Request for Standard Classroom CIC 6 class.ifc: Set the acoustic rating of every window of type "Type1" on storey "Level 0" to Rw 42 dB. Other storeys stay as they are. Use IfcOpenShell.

First a look at what the model holds.

```python
import ifcopenshell
import ifcopenshell.util.element

model = ifcopenshell.open("Standard Classroom CIC 6 class.ifc")
print(model.schema)
storey = next(s for s in model.by_type("IfcBuildingStorey") if s.Name == "Level 0")
windows = [e for e in ifcopenshell.util.element.get_decomposition(storey) if e.is_a("IfcWindow")]
seen = {}
for e in windows:
    element_type = ifcopenshell.util.element.get_type(e)
    key = (element_type.Name if element_type != e and element_type else None, ifcopenshell.util.element.get_pset(e, "Pset_WindowCommon", "AcousticRating"))
    seen[key] = seen.get(key, 0) + 1
for (name, value), count in sorted(seen.items(), key=str):
    print(count, "x", name, "|", value)
```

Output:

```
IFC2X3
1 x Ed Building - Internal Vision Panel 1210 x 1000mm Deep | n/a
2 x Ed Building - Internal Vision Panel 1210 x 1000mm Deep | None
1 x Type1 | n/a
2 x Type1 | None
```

```python
import ifcopenshell
import ifcopenshell.api.pset
import ifcopenshell.util.element

model = ifcopenshell.open("Standard Classroom CIC 6 class.ifc")

storey = next(s for s in model.by_type("IfcBuildingStorey") if s.Name == "Level 0")
windows = [e for e in ifcopenshell.util.element.get_decomposition(storey) if e.is_a("IfcWindow")]

count = 0
for e in windows:
    element_type = ifcopenshell.util.element.get_type(e)
    if element_type in (None, e) or element_type.Name != "Type1":
        continue
    # add_pset returns the element's existing set when there is one.
    pset = ifcopenshell.api.pset.add_pset(model, product=e, name="Pset_WindowCommon")
    ifcopenshell.api.pset.edit_pset(model, pset=pset, properties={"AcousticRating": "Rw 42 dB"})
    count += 1

print(count, "windows updated")

model.write("Standard Classroom CIC 6 class_updated.ifc")
```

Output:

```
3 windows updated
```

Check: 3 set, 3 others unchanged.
